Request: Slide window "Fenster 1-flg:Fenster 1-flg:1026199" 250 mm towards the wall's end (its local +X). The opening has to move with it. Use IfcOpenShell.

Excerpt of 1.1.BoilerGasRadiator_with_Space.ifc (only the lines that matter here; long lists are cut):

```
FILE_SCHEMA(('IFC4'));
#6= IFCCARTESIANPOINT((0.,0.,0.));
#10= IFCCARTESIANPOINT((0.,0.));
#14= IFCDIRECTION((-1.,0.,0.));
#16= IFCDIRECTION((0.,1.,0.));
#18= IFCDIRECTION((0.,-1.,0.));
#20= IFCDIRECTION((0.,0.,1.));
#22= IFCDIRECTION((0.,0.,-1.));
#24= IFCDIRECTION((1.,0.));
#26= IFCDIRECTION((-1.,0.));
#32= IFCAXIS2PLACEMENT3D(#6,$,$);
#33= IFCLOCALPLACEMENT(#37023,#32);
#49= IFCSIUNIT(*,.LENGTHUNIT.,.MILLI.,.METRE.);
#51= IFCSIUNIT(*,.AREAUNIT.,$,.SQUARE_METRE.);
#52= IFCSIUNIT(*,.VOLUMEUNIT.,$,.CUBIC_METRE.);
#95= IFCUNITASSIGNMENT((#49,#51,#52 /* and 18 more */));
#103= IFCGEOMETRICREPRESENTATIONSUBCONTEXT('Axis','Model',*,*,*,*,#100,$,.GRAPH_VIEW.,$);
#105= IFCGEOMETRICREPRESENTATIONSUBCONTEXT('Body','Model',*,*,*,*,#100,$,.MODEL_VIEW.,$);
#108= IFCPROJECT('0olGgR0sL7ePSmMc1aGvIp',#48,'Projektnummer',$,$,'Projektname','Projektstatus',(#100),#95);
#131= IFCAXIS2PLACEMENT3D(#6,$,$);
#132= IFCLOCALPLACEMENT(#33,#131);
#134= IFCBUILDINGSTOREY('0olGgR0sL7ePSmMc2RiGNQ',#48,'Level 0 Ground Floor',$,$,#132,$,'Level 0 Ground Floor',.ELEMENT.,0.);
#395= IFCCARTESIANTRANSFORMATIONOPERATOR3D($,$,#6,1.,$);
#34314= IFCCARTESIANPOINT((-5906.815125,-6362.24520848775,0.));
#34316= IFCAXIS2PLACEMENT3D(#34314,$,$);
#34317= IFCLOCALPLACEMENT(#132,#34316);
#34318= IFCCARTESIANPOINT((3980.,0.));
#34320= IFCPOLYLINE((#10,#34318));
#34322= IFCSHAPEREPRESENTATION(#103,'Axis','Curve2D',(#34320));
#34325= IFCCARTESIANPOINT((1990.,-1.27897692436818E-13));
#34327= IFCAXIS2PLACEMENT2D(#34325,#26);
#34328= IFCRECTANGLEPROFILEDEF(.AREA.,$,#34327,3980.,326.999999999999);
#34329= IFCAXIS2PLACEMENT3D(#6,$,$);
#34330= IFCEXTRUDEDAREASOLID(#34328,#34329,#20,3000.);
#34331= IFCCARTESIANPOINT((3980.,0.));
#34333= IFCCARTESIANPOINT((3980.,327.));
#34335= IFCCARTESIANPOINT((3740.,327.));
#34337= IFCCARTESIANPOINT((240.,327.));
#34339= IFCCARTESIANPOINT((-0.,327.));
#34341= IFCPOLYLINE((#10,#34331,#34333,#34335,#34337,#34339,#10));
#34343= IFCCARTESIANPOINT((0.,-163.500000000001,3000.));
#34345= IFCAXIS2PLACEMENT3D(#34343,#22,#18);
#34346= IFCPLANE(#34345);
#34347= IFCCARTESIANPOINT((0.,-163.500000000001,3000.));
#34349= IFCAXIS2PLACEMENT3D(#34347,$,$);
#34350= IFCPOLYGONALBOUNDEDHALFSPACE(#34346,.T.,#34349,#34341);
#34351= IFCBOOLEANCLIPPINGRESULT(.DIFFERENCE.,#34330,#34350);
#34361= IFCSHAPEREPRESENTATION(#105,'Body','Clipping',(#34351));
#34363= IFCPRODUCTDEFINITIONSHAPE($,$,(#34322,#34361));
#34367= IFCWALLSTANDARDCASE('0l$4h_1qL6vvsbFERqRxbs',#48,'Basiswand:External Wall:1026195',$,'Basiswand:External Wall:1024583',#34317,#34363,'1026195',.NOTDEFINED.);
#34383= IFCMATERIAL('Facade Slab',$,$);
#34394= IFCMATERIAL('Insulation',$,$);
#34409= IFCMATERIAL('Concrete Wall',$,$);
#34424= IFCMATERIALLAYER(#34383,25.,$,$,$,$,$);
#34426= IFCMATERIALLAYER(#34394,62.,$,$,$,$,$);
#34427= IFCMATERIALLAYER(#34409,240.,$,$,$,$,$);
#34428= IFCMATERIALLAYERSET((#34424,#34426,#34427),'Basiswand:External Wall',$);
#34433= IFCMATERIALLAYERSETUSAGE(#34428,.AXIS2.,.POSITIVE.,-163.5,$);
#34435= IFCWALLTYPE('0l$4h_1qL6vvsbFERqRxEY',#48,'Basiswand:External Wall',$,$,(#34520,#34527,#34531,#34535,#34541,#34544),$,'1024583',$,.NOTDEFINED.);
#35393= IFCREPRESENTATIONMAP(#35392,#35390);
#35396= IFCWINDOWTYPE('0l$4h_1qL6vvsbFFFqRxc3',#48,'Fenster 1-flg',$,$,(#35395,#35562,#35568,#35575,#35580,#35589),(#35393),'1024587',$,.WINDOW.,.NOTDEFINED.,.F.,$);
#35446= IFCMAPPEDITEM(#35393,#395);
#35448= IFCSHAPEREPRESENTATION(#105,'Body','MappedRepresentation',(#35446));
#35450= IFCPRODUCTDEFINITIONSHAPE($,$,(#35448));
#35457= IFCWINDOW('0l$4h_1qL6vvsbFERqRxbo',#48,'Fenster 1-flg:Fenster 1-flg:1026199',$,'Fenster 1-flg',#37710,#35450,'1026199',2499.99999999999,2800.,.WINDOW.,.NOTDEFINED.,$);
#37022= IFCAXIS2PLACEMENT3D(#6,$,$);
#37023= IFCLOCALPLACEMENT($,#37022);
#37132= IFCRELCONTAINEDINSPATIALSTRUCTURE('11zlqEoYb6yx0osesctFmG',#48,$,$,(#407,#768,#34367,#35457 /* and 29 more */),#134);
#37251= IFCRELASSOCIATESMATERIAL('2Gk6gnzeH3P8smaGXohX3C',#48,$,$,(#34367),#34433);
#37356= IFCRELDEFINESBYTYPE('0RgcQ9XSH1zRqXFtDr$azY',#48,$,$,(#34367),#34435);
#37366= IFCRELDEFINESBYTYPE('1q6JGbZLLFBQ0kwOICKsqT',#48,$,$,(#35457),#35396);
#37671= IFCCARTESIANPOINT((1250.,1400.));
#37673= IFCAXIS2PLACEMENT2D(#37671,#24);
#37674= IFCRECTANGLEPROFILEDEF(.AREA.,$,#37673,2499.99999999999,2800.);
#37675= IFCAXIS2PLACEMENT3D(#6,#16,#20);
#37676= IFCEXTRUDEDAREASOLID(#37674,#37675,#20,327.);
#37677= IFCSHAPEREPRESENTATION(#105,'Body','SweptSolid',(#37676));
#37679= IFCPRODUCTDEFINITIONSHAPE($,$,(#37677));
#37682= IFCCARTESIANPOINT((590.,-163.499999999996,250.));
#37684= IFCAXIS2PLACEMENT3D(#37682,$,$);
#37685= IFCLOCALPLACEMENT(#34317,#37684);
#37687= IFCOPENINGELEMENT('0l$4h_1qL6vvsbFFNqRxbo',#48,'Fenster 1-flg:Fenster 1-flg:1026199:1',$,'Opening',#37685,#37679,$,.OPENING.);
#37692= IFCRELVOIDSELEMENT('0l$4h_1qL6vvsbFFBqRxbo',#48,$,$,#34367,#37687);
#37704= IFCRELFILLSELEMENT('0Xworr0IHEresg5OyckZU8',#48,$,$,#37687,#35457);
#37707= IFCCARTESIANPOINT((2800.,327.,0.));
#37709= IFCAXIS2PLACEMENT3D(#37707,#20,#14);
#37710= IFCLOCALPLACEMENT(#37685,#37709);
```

```python
import ifcopenshell
import ifcopenshell.api.geometry
import ifcopenshell.util.placement
import ifcopenshell.util.unit

model = ifcopenshell.open("1.1.BoilerGasRadiator_with_Space.ifc")
unit_scale = ifcopenshell.util.unit.calculate_unit_scale(model)

window = model.by_guid("0l$4h_1qL6vvsbFERqRxbo")
opening = window.FillsVoids[0].RelatingOpeningElement
wall = opening.VoidsElements[0].RelatingBuildingElement

wall_matrix = ifcopenshell.util.placement.get_local_placement(wall.ObjectPlacement)
shift = wall_matrix[:3, 0] * 0.25 / unit_scale
before = ifcopenshell.util.placement.get_local_placement(window.ObjectPlacement)[:3, 3].copy()

# The window is placed relative to its opening, so it follows when the opening moves.
matrix = ifcopenshell.util.placement.get_local_placement(opening.ObjectPlacement)
matrix[:3, 3] += shift
ifcopenshell.api.geometry.edit_object_placement(
    model, product=opening, matrix=matrix, is_si=False, should_transform_children=True
)

after = ifcopenshell.util.placement.get_local_placement(window.ObjectPlacement)[:3, 3]
print("window moved by", (after - before).round(3) + 0.0)

model.write("1.1.BoilerGasRadiator_with_Space_rev.ifc")
```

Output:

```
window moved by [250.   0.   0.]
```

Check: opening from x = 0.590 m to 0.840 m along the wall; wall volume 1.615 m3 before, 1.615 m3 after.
